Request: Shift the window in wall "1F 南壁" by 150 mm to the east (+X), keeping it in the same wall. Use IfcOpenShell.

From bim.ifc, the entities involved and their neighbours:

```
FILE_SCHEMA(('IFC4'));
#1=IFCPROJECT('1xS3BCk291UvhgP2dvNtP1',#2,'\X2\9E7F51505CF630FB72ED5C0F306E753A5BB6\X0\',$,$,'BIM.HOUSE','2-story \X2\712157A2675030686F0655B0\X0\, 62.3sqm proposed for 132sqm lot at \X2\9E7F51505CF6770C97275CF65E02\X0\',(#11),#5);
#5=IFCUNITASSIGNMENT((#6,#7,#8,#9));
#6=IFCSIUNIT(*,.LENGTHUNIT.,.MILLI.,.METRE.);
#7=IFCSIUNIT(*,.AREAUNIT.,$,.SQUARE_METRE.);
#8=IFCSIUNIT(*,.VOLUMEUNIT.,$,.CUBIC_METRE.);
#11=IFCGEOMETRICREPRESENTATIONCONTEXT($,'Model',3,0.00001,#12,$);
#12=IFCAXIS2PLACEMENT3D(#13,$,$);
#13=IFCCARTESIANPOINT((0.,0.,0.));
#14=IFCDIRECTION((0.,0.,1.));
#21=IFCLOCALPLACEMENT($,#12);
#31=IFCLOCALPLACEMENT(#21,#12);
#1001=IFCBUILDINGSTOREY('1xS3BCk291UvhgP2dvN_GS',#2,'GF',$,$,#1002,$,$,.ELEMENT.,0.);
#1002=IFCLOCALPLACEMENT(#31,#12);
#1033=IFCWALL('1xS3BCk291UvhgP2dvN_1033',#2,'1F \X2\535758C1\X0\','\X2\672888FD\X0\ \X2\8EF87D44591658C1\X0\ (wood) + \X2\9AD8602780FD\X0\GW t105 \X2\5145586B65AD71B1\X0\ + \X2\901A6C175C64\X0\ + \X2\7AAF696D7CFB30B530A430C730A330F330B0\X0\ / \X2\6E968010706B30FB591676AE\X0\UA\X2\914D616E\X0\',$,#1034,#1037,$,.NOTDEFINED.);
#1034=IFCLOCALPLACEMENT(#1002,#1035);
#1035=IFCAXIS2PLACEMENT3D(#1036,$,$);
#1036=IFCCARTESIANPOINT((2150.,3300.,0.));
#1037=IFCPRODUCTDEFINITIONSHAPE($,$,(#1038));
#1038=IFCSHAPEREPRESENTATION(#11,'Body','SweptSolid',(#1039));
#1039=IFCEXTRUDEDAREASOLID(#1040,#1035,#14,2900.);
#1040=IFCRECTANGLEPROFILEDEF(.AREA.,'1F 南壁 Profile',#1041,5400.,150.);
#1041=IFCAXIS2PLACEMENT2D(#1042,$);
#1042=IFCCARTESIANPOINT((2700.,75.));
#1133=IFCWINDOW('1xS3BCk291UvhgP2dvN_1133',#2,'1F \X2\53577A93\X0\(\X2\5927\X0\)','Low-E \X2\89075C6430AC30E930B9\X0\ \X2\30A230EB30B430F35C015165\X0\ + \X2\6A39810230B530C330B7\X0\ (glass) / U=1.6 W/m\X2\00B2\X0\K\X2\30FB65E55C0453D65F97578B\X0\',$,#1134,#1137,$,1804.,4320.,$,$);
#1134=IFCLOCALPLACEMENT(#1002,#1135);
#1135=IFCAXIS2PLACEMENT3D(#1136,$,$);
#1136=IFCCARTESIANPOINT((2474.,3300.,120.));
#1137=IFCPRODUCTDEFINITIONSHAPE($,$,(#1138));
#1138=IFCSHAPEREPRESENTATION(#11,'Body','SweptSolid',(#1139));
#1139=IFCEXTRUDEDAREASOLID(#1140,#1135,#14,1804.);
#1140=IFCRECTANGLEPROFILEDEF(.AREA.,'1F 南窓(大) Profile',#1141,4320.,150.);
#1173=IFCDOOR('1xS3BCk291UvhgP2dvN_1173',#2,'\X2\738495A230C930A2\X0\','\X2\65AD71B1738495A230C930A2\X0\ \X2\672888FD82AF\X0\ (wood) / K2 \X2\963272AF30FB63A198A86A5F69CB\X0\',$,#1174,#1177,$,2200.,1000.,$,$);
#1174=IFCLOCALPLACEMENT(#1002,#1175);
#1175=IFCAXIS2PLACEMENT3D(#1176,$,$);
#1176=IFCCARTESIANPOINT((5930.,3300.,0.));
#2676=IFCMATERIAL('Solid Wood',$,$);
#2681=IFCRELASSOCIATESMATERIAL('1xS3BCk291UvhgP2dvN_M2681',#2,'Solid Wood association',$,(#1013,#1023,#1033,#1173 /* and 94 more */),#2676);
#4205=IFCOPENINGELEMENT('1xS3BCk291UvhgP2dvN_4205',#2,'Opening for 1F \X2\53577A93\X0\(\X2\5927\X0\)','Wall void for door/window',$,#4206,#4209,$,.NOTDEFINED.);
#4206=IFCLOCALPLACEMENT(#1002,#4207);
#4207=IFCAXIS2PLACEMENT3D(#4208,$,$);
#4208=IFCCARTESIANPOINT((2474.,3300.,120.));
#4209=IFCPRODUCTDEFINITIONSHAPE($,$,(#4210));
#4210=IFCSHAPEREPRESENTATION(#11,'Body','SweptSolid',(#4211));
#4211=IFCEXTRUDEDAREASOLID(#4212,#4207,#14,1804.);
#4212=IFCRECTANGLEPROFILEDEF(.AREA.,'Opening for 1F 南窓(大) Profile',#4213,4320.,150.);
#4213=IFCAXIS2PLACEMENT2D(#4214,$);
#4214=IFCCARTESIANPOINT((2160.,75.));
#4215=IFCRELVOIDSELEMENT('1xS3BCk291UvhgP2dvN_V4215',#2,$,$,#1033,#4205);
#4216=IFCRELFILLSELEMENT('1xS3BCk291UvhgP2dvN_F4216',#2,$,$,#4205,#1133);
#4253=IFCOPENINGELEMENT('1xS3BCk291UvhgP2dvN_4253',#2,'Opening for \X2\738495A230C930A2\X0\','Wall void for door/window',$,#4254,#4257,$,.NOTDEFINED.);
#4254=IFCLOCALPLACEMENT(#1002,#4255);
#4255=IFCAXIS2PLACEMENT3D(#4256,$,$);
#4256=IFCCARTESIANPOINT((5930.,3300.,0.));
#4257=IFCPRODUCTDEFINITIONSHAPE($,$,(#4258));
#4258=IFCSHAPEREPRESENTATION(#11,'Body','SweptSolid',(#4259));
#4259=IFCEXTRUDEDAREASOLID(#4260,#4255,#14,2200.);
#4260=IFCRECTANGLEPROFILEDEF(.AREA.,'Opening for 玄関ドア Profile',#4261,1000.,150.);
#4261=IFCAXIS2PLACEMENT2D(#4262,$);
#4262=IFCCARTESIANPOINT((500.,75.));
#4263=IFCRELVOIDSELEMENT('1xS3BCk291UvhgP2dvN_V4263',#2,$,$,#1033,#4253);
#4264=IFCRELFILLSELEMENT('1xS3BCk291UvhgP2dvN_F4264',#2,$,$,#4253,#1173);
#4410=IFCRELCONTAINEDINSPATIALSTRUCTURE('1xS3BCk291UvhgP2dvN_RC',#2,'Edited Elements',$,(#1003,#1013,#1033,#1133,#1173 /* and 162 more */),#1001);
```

```python
import ifcopenshell
import ifcopenshell.api.geometry
import ifcopenshell.util.placement

model = ifcopenshell.open("bim.ifc")

window = model.by_guid("1xS3BCk291UvhgP2dvN_1133")
opening = window.FillsVoids[0].RelatingOpeningElement
wall = opening.VoidsElements[0].RelatingBuildingElement

wall_matrix = ifcopenshell.util.placement.get_local_placement(wall.ObjectPlacement)
shift = wall_matrix[:3, 0] * 150.0
before = ifcopenshell.util.placement.get_local_placement(window.ObjectPlacement)[:3, 3].copy()

# The window is not placed relative to its opening, so move both.
for product in (opening, window):
    matrix = ifcopenshell.util.placement.get_local_placement(product.ObjectPlacement)
    matrix[:3, 3] += shift
    ifcopenshell.api.geometry.edit_object_placement(model, product=product, matrix=matrix, is_si=False)

after = ifcopenshell.util.placement.get_local_placement(window.ObjectPlacement)[:3, 3]
print("window moved by", (after - before).round(3) + 0.0)

model.write("bim_rev.ifc")
```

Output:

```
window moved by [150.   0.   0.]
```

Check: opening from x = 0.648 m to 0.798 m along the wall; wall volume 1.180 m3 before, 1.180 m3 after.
